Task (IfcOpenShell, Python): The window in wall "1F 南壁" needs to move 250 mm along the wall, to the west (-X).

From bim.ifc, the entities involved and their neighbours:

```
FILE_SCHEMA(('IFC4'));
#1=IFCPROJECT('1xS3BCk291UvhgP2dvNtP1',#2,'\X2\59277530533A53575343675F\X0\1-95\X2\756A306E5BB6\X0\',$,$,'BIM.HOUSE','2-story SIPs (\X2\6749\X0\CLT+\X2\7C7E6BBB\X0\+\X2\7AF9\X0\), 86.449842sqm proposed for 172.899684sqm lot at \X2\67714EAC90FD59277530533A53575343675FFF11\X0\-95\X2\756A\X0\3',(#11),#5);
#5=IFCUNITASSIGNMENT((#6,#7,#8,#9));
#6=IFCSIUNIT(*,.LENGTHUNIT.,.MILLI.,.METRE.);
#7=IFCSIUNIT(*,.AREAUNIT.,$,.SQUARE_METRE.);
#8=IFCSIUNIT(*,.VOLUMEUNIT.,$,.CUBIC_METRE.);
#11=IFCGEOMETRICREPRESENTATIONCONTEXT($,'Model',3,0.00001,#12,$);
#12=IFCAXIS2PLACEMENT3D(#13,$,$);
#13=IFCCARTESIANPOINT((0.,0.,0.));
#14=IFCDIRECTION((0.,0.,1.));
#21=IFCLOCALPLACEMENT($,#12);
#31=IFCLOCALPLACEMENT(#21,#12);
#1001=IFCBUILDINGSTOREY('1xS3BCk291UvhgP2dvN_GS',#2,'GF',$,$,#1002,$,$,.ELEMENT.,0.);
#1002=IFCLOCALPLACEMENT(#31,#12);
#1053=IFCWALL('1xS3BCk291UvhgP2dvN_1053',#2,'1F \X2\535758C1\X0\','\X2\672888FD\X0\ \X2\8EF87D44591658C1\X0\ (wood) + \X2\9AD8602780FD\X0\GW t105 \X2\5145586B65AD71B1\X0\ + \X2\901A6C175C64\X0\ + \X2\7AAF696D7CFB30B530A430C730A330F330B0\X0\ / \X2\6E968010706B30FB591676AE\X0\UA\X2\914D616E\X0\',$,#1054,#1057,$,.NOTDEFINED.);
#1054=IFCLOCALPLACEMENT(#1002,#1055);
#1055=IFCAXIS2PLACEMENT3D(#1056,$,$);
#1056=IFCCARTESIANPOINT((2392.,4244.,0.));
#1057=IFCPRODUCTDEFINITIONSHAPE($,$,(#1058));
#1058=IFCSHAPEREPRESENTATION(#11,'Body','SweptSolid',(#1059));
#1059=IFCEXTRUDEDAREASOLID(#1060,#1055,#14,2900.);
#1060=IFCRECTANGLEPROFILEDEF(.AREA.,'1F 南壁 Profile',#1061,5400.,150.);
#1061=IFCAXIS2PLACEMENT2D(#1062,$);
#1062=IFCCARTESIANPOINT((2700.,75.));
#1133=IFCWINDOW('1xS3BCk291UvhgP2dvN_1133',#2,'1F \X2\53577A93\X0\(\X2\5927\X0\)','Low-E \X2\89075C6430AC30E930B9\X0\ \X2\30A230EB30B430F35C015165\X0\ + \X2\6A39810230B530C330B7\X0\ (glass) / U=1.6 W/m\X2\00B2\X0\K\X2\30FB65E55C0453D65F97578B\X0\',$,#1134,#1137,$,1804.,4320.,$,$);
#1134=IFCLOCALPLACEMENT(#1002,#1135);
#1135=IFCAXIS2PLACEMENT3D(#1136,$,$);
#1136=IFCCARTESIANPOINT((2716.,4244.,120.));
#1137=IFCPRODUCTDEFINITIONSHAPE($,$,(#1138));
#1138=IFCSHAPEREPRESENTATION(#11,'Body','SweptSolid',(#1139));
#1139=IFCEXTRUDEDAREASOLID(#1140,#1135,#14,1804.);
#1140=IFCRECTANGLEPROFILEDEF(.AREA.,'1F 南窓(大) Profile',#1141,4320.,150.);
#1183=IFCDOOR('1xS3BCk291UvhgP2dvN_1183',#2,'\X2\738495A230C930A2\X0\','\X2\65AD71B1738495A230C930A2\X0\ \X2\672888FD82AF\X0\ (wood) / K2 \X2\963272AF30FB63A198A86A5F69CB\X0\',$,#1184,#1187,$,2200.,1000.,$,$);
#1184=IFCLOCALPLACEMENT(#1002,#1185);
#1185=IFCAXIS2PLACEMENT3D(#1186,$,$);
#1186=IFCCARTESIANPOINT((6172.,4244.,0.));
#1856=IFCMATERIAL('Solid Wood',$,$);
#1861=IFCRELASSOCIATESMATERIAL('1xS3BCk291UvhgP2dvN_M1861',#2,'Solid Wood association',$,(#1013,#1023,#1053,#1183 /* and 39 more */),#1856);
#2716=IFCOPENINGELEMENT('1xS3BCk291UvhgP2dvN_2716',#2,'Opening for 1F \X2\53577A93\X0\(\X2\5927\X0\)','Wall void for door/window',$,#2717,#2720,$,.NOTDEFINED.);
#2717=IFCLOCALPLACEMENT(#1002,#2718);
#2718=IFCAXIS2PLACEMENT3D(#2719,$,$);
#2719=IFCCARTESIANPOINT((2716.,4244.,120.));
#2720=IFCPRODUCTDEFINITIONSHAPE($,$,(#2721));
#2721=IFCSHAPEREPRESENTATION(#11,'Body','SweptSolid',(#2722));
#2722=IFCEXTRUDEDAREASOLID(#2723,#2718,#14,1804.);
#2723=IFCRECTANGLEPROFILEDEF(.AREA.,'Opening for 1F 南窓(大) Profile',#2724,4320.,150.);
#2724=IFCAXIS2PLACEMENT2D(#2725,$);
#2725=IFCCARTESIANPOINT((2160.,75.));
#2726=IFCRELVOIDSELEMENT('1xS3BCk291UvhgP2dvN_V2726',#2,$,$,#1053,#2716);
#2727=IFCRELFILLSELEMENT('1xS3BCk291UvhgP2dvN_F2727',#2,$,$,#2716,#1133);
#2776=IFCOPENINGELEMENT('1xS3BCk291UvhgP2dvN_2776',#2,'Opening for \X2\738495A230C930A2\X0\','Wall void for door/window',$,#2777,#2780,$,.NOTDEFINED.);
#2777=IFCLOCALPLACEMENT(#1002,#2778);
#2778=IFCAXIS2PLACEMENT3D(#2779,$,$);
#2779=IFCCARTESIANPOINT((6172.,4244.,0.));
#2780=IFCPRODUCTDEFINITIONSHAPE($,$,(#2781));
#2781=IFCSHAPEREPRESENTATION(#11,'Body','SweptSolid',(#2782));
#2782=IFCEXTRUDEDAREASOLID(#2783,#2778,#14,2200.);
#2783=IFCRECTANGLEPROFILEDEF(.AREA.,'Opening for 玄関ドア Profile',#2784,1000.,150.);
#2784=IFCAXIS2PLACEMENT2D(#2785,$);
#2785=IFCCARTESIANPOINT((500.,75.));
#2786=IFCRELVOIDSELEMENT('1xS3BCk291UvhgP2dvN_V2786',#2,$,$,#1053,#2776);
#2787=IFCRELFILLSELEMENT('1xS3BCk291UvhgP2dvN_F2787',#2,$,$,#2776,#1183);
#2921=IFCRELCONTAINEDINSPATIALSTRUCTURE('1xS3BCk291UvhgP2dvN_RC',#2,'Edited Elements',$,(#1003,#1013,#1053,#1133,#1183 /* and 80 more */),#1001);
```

```python
import ifcopenshell
import ifcopenshell.api.geometry
import ifcopenshell.util.placement
import ifcopenshell.util.unit

model = ifcopenshell.open("bim.ifc")
unit_scale = ifcopenshell.util.unit.calculate_unit_scale(model)

window = model.by_guid("1xS3BCk291UvhgP2dvN_1133")
opening = window.FillsVoids[0].RelatingOpeningElement
wall = opening.VoidsElements[0].RelatingBuildingElement

wall_matrix = ifcopenshell.util.placement.get_local_placement(wall.ObjectPlacement)
shift = wall_matrix[:3, 0] * -0.25 / unit_scale
before = ifcopenshell.util.placement.get_local_placement(window.ObjectPlacement)[:3, 3].copy()

# The window is not placed relative to its opening, so move both.
for product in (opening, window):
    matrix = ifcopenshell.util.placement.get_local_placement(product.ObjectPlacement)
    matrix[:3, 3] += shift
    ifcopenshell.api.geometry.edit_object_placement(model, product=product, matrix=matrix, is_si=False)

after = ifcopenshell.util.placement.get_local_placement(window.ObjectPlacement)[:3, 3]
print("window moved by", (after - before).round(3) + 0.0)

model.write("bim_rev.ifc")
```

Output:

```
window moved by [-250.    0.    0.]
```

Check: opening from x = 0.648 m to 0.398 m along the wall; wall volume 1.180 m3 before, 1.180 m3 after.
